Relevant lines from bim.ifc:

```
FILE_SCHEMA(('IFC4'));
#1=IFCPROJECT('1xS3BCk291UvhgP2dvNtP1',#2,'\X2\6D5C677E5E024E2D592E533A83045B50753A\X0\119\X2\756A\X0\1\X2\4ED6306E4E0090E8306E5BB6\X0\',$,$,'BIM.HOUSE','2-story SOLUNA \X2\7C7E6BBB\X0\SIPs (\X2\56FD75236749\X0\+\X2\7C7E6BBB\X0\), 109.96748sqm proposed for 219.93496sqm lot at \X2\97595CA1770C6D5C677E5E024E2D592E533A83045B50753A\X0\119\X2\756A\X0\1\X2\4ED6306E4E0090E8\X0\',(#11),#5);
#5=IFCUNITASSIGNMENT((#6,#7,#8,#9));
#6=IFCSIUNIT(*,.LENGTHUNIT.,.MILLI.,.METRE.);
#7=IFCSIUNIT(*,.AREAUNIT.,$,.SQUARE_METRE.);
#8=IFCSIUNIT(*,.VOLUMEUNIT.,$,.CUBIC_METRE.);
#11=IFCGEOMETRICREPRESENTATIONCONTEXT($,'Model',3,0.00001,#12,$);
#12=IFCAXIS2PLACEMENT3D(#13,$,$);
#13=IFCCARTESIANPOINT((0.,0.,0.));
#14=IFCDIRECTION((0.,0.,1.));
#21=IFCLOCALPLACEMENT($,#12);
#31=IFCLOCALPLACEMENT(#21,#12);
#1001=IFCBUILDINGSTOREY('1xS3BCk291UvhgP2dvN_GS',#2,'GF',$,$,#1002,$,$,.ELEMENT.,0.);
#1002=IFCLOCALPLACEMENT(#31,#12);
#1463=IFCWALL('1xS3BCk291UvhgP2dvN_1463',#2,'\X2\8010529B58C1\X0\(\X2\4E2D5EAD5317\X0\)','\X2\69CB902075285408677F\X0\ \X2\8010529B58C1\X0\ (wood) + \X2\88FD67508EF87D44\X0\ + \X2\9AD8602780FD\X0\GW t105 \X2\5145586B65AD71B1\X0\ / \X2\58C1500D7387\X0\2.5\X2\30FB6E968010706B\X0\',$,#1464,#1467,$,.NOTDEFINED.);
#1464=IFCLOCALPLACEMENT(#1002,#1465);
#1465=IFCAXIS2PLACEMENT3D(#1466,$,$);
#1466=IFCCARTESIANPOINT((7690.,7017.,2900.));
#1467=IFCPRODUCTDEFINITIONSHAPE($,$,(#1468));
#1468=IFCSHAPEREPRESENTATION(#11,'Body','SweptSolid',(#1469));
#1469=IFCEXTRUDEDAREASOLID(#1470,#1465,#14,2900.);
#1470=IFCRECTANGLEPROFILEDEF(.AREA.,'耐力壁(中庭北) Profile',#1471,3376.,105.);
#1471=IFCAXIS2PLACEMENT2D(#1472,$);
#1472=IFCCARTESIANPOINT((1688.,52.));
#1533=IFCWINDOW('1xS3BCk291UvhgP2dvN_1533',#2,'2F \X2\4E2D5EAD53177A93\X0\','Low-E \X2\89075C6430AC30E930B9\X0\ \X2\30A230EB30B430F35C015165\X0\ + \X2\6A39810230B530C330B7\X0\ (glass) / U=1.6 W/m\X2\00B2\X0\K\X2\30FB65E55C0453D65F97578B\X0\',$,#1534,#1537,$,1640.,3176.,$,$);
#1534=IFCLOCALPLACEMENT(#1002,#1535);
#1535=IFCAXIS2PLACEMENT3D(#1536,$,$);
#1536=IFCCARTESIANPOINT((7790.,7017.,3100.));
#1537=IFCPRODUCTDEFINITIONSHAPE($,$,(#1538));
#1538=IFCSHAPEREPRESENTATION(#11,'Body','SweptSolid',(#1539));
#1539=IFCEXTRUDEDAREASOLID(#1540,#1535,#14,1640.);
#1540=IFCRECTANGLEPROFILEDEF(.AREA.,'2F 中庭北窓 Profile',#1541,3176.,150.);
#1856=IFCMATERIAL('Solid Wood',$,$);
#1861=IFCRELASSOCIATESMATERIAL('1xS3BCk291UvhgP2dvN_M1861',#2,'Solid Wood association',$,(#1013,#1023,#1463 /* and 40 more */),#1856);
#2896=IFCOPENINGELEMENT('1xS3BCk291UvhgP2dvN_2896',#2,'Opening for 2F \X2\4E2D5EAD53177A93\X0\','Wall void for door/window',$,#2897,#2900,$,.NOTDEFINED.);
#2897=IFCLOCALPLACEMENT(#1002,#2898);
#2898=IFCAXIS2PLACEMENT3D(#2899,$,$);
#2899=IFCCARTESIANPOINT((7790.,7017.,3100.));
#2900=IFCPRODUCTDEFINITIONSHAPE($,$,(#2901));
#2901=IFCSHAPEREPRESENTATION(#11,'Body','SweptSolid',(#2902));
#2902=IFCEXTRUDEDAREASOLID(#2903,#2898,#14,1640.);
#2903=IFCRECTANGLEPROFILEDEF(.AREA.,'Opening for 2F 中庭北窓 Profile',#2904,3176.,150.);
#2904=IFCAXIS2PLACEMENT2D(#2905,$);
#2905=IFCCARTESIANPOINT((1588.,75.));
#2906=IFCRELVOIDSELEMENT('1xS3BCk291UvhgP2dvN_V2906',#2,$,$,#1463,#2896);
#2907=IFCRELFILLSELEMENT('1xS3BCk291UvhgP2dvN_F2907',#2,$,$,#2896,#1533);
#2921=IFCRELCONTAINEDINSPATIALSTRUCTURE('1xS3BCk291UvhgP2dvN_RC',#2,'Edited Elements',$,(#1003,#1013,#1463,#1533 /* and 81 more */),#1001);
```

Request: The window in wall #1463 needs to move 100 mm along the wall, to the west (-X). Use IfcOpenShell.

```python
import ifcopenshell
import ifcopenshell.api.geometry
import ifcopenshell.util.placement
import ifcopenshell.util.unit

model = ifcopenshell.open("bim.ifc")
unit_scale = ifcopenshell.util.unit.calculate_unit_scale(model)

window = model.by_id(1533)
opening = window.FillsVoids[0].RelatingOpeningElement
wall = opening.VoidsElements[0].RelatingBuildingElement

wall_matrix = ifcopenshell.util.placement.get_local_placement(wall.ObjectPlacement)
shift = wall_matrix[:3, 0] * -0.1 / unit_scale
before = ifcopenshell.util.placement.get_local_placement(window.ObjectPlacement)[:3, 3].copy()

# The window is not placed relative to its opening, so move both.
for product in (opening, window):
    matrix = ifcopenshell.util.placement.get_local_placement(product.ObjectPlacement)
    matrix[:3, 3] += shift
    ifcopenshell.api.geometry.edit_object_placement(model, product=product, matrix=matrix, is_si=False)

after = ifcopenshell.util.placement.get_local_placement(window.ObjectPlacement)[:3, 3]
print("window moved by", (after - before).round(3) + 0.0)

model.write("bim-out.ifc")
```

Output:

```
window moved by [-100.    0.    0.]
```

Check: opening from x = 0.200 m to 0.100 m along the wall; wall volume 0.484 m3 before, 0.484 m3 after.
